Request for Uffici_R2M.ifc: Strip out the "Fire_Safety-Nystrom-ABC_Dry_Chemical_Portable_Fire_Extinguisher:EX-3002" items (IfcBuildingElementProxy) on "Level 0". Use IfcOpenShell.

First a look at what the model holds.

```python
import ifcopenshell
import ifcopenshell.util.element

model = ifcopenshell.open("Uffici_R2M.ifc")
print(model.schema)
storey = next(s for s in model.by_type("IfcBuildingStorey") if s.Name == "Level 0")
proxies = [e for e in ifcopenshell.util.element.get_decomposition(storey) if e.is_a("IfcBuildingElementProxy")]
seen = {}
for e in proxies:
    element_type = ifcopenshell.util.element.get_type(e)
    name = element_type.Name if element_type not in (None, e) else None
    seen[name] = seen.get(name, 0) + 1
for name, count in sorted(seen.items(), key=str):
    print(count, "x", name)
```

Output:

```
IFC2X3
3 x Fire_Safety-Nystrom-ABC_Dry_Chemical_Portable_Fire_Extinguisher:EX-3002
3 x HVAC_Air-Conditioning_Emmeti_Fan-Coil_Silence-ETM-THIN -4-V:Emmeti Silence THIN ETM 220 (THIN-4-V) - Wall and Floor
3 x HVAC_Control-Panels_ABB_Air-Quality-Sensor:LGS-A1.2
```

```python
import ifcopenshell
import ifcopenshell.api.root
import ifcopenshell.util.element

model = ifcopenshell.open("Uffici_R2M.ifc")

storey = next(s for s in model.by_type("IfcBuildingStorey") if s.Name == "Level 0")
proxies = [e for e in ifcopenshell.util.element.get_decomposition(storey) if e.is_a("IfcBuildingElementProxy")]
targets = [e for e in proxies if (t := ifcopenshell.util.element.get_type(e)) not in (None, e) and t.Name == "Fire_Safety-Nystrom-ABC_Dry_Chemical_Portable_Fire_Extinguisher:EX-3002"]

for e in targets:
    ifcopenshell.api.root.remove_product(model, product=e)
print(len(targets), "removed")

model.write("Uffici_R2M_edited.ifc")
```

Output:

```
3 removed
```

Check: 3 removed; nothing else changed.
